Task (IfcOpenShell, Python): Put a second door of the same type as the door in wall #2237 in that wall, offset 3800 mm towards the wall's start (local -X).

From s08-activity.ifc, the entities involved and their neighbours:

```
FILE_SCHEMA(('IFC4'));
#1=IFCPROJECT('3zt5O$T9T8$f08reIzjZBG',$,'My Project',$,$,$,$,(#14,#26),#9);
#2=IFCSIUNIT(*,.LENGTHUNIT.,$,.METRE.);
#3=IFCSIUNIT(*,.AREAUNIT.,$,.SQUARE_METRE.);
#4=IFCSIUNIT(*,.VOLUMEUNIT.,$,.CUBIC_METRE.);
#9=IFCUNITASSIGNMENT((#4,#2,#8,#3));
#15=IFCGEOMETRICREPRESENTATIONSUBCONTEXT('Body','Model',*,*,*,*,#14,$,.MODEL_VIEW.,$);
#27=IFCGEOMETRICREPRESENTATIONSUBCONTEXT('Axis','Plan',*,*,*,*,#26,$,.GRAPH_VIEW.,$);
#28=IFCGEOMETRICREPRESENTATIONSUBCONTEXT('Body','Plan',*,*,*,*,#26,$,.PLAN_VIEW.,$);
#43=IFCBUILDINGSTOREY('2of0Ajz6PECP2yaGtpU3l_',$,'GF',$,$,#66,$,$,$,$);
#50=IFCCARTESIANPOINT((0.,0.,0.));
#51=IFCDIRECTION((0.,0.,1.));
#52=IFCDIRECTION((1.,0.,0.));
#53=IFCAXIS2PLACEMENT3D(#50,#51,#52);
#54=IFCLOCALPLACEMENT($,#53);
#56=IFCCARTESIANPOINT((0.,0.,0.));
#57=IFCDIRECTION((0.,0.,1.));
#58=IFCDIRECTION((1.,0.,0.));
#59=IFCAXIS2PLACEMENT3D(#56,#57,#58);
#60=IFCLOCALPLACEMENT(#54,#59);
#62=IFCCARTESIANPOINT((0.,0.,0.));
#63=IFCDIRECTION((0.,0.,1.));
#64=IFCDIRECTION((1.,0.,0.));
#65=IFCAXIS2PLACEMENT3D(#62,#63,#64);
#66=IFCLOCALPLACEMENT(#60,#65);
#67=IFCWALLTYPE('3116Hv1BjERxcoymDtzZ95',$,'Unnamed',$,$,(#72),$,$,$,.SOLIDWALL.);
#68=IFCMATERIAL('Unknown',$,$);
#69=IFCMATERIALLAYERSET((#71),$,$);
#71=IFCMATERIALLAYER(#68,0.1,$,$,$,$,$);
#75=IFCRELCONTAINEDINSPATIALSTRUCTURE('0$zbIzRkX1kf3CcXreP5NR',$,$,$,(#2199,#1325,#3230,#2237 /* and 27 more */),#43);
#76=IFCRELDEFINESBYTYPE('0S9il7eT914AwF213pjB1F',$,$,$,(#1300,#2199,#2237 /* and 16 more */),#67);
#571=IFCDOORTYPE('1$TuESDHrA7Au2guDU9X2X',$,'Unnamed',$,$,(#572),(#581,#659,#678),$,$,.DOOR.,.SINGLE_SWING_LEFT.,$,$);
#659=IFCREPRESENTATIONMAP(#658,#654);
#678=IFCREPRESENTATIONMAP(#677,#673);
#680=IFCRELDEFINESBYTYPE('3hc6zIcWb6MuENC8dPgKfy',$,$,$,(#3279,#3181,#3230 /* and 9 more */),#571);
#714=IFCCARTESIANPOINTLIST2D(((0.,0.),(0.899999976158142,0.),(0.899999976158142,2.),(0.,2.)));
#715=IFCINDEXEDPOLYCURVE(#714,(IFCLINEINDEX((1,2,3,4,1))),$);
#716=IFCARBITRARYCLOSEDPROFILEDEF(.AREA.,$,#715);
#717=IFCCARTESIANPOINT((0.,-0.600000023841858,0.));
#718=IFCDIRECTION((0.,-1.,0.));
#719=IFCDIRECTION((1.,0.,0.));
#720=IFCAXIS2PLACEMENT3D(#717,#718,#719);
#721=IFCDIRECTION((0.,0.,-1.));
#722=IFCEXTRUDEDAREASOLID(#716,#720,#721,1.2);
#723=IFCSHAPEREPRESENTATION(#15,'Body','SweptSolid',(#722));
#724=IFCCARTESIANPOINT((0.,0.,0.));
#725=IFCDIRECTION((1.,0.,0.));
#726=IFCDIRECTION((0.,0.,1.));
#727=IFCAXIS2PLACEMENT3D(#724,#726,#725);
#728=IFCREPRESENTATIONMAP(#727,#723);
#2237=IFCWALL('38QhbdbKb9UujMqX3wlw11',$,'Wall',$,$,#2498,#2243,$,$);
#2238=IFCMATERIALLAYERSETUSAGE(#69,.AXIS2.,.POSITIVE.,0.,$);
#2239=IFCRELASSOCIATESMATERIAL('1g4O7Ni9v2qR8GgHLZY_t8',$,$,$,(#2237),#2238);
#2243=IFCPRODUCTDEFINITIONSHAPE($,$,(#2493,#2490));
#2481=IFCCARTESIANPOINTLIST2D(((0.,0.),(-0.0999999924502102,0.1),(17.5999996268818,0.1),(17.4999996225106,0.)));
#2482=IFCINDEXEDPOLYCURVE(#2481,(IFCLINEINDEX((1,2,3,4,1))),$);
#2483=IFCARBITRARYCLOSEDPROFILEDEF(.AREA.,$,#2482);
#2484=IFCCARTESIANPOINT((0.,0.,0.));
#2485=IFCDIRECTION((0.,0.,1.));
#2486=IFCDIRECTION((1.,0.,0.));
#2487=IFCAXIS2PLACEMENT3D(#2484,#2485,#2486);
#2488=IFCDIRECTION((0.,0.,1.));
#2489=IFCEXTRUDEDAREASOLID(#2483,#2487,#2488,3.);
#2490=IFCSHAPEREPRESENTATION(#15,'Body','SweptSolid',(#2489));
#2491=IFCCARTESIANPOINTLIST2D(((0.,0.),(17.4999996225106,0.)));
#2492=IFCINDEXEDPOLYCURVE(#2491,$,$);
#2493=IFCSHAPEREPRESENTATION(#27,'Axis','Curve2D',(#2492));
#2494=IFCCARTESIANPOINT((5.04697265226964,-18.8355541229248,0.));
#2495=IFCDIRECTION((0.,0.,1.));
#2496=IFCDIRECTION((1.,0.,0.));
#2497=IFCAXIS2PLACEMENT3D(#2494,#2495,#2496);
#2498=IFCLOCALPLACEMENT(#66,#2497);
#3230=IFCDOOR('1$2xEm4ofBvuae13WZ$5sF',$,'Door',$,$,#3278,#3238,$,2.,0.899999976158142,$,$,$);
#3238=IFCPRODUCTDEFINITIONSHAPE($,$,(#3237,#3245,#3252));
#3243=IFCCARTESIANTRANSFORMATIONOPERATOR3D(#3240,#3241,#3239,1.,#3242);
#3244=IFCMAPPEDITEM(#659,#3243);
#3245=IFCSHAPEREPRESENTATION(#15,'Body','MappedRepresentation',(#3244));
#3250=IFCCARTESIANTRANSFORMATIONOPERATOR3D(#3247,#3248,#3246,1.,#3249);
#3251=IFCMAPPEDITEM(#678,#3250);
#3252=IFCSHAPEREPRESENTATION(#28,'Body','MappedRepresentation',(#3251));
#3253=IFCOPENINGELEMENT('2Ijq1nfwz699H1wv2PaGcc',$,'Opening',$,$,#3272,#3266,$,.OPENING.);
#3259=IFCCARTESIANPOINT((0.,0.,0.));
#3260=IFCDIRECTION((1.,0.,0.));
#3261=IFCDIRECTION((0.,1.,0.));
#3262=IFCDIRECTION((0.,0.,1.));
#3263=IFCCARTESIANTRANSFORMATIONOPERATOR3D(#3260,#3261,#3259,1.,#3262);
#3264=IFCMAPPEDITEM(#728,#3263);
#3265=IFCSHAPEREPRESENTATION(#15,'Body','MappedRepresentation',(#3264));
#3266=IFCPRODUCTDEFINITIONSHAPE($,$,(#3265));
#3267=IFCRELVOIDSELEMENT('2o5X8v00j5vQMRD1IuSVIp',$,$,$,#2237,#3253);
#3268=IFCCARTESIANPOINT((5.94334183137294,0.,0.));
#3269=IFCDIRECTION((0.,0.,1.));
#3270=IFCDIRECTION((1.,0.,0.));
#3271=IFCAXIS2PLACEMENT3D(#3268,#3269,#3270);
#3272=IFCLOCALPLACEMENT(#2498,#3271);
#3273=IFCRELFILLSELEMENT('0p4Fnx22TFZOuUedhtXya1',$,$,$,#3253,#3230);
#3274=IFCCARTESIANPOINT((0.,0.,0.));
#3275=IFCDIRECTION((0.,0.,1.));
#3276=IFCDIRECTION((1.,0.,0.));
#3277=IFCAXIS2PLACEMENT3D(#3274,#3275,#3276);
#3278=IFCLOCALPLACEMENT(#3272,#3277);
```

```python
import ifcopenshell
import ifcopenshell.api.feature
import ifcopenshell.api.geometry
import ifcopenshell.api.root
import ifcopenshell.geom
import ifcopenshell.util.element
import ifcopenshell.util.placement
import ifcopenshell.util.shape
import ifcopenshell.util.unit

model = ifcopenshell.open("s08-activity.ifc")
unit_scale = ifcopenshell.util.unit.calculate_unit_scale(model)
settings = ifcopenshell.geom.settings()


def volume(element):
    """Net volume in cubic metres, openings subtracted."""
    shape = ifcopenshell.geom.create_shape(settings, element)
    return ifcopenshell.util.shape.get_volume(shape.geometry)


door = model.by_guid("1$2xEm4ofBvuae13WZ$5sF")
opening = door.FillsVoids[0].RelatingOpeningElement
wall = opening.VoidsElements[0].RelatingBuildingElement
before = volume(wall)
shift = ifcopenshell.util.placement.get_local_placement(wall.ObjectPlacement)[:3, 0] * -3.8 / unit_scale

# copy_class copies the void relationship, type, container and properties, but no geometry.
new_opening = ifcopenshell.api.root.copy_class(model, product=opening)
new_opening.Representation = ifcopenshell.util.element.copy_deep(
    model, opening.Representation, exclude=["IfcGeometricRepresentationContext", "IfcRepresentationMap"]
)
new_door = ifcopenshell.api.root.copy_class(model, product=door)
new_door.Representation = ifcopenshell.util.element.copy_deep(
    model, door.Representation, exclude=["IfcGeometricRepresentationContext", "IfcRepresentationMap"]
)
ifcopenshell.api.feature.add_filling(model, opening=new_opening, element=new_door)

for old, new in ((opening, new_opening), (door, new_door)):
    matrix = ifcopenshell.util.placement.get_local_placement(old.ObjectPlacement)
    matrix[:3, 3] += shift
    ifcopenshell.api.geometry.edit_object_placement(model, product=new, matrix=matrix, is_si=False)

after = volume(wall)

print(f"wall volume {before:.3f} -> {after:.3f} m3")

model.write("s08-activity-out.ifc")
```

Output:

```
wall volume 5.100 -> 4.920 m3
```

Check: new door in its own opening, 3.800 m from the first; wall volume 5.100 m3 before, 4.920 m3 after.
